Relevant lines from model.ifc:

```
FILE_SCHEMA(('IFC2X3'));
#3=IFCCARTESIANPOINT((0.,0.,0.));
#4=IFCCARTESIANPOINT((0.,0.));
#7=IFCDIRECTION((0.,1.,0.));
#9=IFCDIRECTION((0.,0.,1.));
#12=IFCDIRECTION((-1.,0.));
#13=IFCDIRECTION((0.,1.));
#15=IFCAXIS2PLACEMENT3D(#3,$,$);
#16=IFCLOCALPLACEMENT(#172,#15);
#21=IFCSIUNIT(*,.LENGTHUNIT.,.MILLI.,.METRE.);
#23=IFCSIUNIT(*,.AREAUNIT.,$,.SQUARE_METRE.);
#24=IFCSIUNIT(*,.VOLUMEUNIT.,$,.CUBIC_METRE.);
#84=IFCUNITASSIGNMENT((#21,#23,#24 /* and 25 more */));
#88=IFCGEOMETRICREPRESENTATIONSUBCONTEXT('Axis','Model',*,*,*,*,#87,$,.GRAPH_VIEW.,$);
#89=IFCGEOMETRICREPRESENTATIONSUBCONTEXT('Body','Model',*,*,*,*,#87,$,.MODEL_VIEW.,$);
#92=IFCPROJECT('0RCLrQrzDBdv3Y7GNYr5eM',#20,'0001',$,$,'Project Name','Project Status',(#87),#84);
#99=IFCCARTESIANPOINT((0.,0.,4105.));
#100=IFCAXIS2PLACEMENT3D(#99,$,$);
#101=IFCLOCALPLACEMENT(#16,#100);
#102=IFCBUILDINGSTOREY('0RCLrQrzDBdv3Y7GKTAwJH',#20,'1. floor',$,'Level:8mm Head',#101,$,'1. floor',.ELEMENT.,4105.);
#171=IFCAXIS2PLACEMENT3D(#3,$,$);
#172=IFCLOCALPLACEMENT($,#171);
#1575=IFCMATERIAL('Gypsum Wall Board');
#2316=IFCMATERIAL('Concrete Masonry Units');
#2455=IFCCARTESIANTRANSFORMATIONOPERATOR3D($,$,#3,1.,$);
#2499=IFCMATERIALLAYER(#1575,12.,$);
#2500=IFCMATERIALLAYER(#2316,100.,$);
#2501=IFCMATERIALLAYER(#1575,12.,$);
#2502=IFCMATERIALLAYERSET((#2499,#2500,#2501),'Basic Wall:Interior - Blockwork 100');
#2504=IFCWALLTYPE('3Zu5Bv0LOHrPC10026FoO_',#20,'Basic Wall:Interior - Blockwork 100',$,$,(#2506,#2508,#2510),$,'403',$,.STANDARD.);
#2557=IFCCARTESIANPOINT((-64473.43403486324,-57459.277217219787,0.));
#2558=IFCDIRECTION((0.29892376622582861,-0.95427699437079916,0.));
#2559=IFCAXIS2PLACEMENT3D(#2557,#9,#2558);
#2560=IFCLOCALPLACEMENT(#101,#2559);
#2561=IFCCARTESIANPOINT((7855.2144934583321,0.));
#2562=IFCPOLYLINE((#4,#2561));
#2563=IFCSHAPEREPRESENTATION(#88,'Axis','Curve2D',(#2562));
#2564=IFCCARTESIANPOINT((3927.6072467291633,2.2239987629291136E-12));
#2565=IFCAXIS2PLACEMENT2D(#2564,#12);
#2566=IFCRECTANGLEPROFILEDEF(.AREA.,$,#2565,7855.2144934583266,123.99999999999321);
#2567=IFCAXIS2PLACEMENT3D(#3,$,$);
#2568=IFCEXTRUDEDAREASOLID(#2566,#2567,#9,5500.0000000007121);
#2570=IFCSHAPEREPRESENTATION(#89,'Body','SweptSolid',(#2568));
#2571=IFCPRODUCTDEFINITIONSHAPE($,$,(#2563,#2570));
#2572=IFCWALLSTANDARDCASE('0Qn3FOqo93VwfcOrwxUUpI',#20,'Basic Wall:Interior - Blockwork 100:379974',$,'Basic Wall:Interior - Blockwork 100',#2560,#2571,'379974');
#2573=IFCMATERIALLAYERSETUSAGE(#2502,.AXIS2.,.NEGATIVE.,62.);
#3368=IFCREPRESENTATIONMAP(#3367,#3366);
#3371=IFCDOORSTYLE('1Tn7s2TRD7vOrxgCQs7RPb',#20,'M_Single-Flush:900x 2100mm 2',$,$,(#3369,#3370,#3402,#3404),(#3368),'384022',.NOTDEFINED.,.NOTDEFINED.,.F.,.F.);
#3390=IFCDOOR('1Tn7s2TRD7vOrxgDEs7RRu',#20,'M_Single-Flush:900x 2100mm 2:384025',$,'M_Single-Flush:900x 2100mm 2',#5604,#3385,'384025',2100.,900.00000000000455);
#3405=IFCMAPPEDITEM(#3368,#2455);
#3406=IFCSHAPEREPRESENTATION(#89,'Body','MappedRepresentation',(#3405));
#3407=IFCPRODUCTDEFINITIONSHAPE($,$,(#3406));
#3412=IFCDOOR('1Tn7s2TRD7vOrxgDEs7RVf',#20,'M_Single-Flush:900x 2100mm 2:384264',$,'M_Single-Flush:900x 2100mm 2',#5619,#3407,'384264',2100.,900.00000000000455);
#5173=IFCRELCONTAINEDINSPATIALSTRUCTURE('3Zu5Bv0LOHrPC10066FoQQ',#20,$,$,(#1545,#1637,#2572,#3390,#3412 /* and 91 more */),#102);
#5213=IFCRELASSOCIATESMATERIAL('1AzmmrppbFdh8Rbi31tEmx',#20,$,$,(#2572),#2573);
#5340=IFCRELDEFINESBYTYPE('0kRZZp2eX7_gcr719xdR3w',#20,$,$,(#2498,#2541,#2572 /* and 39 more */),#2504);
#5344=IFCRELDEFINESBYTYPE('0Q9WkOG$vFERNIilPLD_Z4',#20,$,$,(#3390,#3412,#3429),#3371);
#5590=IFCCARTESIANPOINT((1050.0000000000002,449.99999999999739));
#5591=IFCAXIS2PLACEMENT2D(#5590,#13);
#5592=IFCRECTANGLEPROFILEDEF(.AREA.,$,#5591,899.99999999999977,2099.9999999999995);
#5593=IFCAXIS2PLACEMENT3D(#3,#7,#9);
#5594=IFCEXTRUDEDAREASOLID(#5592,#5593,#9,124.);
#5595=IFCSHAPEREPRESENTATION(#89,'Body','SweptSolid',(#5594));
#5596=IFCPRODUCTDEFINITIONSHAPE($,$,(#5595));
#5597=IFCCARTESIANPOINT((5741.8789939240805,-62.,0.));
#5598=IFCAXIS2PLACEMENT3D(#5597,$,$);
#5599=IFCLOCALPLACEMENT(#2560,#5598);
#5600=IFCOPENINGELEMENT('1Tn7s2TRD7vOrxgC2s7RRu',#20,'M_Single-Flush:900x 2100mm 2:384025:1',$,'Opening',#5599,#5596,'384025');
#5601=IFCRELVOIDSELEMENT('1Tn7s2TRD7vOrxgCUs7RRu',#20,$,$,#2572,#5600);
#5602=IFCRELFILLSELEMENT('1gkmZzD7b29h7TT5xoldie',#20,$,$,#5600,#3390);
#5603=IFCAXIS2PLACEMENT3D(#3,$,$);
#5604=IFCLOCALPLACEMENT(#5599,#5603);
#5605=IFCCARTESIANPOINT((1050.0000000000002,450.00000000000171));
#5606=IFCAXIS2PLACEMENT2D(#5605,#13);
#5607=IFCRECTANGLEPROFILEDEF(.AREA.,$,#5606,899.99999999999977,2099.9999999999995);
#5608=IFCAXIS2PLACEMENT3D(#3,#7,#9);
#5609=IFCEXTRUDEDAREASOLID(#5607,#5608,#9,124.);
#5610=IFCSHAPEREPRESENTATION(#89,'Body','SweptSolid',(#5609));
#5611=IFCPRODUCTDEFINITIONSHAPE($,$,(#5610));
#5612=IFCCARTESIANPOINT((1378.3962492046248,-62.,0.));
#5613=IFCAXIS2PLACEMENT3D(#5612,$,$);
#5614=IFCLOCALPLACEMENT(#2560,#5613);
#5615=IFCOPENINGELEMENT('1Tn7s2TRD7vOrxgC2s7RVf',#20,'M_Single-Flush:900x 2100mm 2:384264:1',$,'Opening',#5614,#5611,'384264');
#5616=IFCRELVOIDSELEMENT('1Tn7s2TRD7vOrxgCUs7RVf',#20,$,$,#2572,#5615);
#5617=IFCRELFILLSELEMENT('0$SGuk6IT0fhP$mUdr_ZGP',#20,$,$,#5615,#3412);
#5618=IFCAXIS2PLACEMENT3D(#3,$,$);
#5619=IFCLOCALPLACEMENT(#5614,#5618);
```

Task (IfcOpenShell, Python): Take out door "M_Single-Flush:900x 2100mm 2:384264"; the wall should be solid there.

```python
import ifcopenshell
import ifcopenshell.api.feature
import ifcopenshell.api.root
import ifcopenshell.geom
import ifcopenshell.util.shape

model = ifcopenshell.open("model.ifc")
settings = ifcopenshell.geom.settings()


def volume(element):
    """Net volume in cubic metres, openings subtracted."""
    shape = ifcopenshell.geom.create_shape(settings, element)
    return ifcopenshell.util.shape.get_volume(shape.geometry)


door = model.by_guid("1Tn7s2TRD7vOrxgDEs7RVf")
opening = door.FillsVoids[0].RelatingOpeningElement
wall = opening.VoidsElements[0].RelatingBuildingElement
before = volume(wall)

ifcopenshell.api.root.remove_product(model, product=door)
ifcopenshell.api.feature.remove_feature(model, feature=opening)

after = volume(wall)

print(f"wall volume {before:.3f} -> {after:.3f} m3")

model.write("model_updated.ifc")
```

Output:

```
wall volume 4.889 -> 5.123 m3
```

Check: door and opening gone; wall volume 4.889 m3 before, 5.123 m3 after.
